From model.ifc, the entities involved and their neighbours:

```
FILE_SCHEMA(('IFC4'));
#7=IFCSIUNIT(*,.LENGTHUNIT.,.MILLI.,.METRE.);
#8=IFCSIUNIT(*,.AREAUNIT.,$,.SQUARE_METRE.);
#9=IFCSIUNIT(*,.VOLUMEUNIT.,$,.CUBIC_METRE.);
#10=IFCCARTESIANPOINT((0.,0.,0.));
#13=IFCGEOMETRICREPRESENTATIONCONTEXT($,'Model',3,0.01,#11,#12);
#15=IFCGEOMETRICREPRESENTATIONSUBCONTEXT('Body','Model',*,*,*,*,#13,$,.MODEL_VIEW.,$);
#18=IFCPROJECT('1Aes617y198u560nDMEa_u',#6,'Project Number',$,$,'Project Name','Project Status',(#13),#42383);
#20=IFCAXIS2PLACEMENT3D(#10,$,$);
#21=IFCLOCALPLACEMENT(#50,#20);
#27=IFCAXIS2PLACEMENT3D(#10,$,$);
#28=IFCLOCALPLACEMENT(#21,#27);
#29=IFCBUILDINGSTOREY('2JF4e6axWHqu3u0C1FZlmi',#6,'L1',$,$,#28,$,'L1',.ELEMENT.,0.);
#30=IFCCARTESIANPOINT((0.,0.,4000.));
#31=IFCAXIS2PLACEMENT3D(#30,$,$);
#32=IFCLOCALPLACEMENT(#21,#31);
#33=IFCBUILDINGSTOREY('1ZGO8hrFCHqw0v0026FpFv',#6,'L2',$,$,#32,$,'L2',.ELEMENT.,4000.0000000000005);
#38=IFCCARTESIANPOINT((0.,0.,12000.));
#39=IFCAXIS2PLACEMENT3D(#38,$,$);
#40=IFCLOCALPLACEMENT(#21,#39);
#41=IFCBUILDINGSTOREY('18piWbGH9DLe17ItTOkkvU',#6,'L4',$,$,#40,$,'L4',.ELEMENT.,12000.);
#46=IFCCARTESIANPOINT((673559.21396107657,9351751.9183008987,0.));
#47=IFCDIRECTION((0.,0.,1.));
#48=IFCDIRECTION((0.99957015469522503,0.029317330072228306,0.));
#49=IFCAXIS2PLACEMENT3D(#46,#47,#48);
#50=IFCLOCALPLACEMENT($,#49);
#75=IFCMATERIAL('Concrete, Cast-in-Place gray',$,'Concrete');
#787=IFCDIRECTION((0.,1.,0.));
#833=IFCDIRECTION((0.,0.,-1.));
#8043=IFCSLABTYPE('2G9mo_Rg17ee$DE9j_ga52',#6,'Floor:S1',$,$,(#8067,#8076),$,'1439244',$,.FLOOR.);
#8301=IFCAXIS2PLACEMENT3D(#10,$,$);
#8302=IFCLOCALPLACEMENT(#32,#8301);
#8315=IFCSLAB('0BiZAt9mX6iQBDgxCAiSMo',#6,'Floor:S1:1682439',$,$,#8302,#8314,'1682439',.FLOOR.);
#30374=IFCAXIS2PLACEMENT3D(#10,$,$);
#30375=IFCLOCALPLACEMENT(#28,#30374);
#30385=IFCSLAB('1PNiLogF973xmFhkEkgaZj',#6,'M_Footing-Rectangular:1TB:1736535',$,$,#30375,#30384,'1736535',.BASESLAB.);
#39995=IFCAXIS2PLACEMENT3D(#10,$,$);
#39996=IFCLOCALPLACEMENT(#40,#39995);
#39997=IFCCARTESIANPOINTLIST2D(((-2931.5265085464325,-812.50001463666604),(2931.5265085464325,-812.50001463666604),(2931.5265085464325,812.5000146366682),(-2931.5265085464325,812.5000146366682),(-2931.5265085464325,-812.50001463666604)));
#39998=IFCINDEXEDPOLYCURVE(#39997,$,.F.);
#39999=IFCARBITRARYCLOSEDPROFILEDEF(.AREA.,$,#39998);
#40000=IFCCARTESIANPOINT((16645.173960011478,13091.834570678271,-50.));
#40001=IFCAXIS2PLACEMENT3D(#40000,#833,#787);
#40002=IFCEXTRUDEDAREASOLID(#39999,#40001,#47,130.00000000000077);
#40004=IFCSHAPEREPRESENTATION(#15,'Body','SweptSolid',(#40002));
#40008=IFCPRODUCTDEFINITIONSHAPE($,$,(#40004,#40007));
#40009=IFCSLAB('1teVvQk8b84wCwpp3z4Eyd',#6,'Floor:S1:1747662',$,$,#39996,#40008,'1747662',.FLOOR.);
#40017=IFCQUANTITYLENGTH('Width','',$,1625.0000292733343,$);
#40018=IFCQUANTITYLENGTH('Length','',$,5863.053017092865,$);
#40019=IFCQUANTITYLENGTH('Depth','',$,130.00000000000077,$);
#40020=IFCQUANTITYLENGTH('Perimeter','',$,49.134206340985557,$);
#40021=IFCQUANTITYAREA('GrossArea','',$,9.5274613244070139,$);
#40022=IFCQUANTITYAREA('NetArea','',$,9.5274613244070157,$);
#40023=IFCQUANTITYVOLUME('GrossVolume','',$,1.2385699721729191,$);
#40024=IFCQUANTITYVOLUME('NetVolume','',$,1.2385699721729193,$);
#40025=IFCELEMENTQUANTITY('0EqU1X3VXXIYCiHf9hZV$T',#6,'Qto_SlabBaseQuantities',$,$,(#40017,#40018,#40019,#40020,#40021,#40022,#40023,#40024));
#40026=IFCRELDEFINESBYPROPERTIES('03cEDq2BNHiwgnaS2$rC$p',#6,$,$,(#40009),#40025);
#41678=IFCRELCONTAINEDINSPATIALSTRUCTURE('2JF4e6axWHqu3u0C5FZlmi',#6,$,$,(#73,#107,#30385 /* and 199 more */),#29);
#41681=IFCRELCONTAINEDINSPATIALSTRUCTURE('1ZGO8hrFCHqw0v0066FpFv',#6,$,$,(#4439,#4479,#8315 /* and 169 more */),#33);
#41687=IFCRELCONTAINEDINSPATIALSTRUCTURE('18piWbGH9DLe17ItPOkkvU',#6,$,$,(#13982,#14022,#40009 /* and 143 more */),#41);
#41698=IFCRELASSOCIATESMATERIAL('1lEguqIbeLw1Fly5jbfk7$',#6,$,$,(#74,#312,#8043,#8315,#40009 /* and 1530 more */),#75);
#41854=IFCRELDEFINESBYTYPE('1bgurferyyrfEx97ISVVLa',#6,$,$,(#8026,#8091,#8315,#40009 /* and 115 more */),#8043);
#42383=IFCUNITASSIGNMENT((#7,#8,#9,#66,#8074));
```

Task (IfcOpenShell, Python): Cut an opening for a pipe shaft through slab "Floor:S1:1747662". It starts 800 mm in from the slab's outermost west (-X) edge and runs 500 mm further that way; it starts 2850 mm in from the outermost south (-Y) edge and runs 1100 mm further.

```python
import numpy as np
import ifcopenshell
import ifcopenshell.api.feature
import ifcopenshell.api.geometry
import ifcopenshell.api.pset
import ifcopenshell.api.root
import ifcopenshell.geom
import ifcopenshell.util.element
import ifcopenshell.util.placement
import ifcopenshell.util.representation
import ifcopenshell.util.shape
import ifcopenshell.util.unit

model = ifcopenshell.open("model.ifc")
unit_scale = ifcopenshell.util.unit.calculate_unit_scale(model)
area_scale = ifcopenshell.util.unit.calculate_unit_scale(model, "AREAUNIT")
volume_scale = ifcopenshell.util.unit.calculate_unit_scale(model, "VOLUMEUNIT")
settings = ifcopenshell.geom.settings()


def volume(element):
    """Net volume in cubic metres, openings subtracted."""
    shape = ifcopenshell.geom.create_shape(settings, element)
    return ifcopenshell.util.shape.get_volume(shape.geometry)


slab = model.by_guid("1teVvQk8b84wCwpp3z4Eyd")
before = volume(slab)

# Extent in the slab's own axes, in metres. The edges named are its -X and -Y sides.
slab_shape = ifcopenshell.geom.create_shape(settings, slab)
vertices = ifcopenshell.util.shape.get_vertices(slab_shape.geometry)
x_min, y_min, bottom = vertices.min(axis=0)
top = vertices[:, 2].max()

opening = ifcopenshell.api.root.create_entity(model, ifc_class="IfcOpeningElement", name="Pipe shaft opening", predefined_type="OPENING")
context = ifcopenshell.util.representation.get_context(model, "Model", "Body", "MODEL_VIEW")
width, depth = 0.5, 1.1
outline = [(0.0, 0.0), (width, 0.0), (width, depth), (0.0, depth), (0.0, 0.0)]
# Overshoot both faces by 50 mm so the cut is clean.
shape = ifcopenshell.api.geometry.add_slab_representation(
    model, context=context, depth=top - bottom + 0.1, polyline=outline
)
ifcopenshell.api.geometry.assign_representation(model, product=opening, representation=shape)

matrix = ifcopenshell.util.placement.get_local_placement(slab.ObjectPlacement)
matrix[:, 3] = matrix @ np.append(np.array([x_min + 0.8, y_min + 2.85, bottom - 0.05]) / unit_scale, 1.0)
ifcopenshell.api.geometry.edit_object_placement(model, product=opening, matrix=matrix, is_si=False)
ifcopenshell.api.feature.add_feature(model, feature=opening, element=slab)

after = volume(slab)

# Update the slab's stored quantities.
qto = model.by_id(ifcopenshell.util.element.get_pset(slab, "Qto_SlabBaseQuantities", should_inherit=False)["id"])
ifcopenshell.api.pset.edit_qto(model, qto=qto, properties={
    "NetArea": after / (top - bottom) / area_scale,
    "NetVolume": after / volume_scale,
})

print(f"slab volume {before:.3f} -> {after:.3f} m3")

model.write("model_edited.ifc")
```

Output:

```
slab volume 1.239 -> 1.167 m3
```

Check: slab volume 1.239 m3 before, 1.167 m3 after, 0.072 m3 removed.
